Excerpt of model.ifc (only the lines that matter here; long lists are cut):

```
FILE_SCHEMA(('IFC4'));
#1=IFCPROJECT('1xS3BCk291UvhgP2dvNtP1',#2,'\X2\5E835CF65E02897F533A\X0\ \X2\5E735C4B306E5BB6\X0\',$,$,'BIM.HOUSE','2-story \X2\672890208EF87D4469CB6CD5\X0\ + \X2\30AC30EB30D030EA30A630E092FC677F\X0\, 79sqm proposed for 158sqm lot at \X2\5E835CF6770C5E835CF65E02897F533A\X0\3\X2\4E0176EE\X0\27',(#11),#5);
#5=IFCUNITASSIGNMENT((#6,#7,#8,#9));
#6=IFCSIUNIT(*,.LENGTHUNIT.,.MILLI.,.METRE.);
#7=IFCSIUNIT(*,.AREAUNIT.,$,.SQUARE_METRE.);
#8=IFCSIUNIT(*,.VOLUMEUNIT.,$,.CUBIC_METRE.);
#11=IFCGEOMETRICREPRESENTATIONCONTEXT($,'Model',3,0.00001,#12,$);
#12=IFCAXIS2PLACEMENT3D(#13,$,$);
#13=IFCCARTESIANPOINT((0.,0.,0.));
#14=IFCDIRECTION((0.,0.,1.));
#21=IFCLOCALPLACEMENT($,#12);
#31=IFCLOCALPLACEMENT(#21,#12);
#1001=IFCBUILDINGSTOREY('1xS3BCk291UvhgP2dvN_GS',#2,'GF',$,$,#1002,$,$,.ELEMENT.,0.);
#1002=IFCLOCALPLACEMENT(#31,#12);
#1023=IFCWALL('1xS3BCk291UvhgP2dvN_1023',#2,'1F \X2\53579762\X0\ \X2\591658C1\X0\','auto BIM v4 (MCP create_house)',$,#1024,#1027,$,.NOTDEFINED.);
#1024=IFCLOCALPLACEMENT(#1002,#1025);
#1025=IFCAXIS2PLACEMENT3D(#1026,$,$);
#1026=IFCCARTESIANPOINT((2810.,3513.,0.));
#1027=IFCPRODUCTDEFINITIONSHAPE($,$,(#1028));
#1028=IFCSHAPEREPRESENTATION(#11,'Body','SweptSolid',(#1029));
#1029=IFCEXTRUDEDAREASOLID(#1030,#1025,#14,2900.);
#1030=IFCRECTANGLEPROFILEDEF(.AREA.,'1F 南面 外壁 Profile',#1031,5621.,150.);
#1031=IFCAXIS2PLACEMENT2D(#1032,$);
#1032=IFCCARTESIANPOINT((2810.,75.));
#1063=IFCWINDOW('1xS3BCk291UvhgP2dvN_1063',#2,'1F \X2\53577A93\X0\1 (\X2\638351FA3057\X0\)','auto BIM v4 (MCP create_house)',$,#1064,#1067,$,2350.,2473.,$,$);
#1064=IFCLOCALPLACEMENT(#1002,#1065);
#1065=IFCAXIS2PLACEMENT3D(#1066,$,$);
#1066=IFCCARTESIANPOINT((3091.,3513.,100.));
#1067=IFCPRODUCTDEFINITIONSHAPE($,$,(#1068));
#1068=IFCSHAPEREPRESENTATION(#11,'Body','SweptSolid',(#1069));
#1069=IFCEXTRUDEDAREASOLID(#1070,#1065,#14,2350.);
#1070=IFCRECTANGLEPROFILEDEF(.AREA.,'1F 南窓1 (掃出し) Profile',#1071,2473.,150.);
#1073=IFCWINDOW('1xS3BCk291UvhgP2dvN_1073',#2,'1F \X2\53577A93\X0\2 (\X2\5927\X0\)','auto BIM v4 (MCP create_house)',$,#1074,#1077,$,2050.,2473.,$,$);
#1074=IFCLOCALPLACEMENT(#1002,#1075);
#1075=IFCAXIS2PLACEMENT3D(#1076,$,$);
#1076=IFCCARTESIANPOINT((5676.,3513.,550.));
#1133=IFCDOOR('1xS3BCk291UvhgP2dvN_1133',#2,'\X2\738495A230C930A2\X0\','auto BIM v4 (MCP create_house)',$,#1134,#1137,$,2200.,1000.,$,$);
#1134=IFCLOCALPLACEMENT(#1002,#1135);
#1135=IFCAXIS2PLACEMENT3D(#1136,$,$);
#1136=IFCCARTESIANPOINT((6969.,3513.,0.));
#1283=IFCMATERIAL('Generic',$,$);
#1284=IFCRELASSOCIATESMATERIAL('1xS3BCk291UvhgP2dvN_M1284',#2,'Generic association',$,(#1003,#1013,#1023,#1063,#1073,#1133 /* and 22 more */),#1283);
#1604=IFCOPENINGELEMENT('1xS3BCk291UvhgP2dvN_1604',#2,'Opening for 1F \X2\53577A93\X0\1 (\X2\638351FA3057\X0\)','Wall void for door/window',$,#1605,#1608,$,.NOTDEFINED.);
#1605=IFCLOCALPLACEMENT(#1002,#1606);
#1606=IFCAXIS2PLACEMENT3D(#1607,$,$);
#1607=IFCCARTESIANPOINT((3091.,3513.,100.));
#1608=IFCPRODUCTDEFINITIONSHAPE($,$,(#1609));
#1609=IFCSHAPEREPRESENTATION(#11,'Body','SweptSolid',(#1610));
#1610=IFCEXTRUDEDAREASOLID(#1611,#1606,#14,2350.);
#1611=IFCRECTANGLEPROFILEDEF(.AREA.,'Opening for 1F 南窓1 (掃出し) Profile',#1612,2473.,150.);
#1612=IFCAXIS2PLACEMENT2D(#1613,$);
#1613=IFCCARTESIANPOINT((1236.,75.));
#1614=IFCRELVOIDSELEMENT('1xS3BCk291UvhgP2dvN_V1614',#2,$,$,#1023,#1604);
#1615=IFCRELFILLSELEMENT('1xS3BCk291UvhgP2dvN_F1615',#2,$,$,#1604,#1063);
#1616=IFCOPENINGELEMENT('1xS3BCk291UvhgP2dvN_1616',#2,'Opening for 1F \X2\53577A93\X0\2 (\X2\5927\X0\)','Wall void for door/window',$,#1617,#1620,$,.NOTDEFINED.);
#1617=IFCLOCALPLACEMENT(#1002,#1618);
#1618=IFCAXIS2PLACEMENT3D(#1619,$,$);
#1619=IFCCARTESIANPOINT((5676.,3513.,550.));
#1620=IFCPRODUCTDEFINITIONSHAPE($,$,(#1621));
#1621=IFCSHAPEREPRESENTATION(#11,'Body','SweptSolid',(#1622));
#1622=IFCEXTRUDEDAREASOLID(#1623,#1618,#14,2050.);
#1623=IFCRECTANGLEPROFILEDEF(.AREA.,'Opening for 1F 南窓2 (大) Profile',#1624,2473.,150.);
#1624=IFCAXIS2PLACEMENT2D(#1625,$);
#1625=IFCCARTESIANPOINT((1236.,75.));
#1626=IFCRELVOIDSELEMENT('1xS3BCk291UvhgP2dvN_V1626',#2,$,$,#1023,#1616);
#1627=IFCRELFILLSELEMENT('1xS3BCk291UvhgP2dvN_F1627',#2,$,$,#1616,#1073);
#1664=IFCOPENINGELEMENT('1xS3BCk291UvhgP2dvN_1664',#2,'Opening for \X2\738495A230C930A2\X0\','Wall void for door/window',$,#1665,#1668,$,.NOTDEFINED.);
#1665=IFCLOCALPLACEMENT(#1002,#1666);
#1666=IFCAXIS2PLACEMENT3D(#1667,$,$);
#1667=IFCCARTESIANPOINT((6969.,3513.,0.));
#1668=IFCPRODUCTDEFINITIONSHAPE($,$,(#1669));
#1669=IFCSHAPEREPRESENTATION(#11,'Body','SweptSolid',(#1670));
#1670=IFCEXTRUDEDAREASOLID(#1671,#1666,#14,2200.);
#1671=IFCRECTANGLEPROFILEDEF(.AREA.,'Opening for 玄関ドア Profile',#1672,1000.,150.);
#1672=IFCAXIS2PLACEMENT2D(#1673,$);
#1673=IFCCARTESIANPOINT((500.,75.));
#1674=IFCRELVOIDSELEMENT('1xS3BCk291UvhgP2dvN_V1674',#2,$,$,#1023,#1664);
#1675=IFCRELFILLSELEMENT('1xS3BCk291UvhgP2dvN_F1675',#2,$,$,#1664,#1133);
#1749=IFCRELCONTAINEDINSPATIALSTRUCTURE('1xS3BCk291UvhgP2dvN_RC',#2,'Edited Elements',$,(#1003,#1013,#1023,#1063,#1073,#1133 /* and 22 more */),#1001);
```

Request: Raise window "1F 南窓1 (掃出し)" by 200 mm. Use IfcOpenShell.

```python
import numpy as np
import ifcopenshell
import ifcopenshell.api.geometry
import ifcopenshell.util.placement
import ifcopenshell.util.unit

model = ifcopenshell.open("model.ifc")
unit_scale = ifcopenshell.util.unit.calculate_unit_scale(model)

window = model.by_guid("1xS3BCk291UvhgP2dvN_1063")
opening = window.FillsVoids[0].RelatingOpeningElement
dz = 200.0

shift = np.array([0.0, 0.0, dz])
# The window is not placed relative to its opening, so move both.
for product in (opening, window):
    matrix = ifcopenshell.util.placement.get_local_placement(product.ObjectPlacement)
    matrix[:3, 3] += shift
    ifcopenshell.api.geometry.edit_object_placement(model, product=product, matrix=matrix, is_si=False)

print(f"moved by {dz * unit_scale:+.3f} m")

model.write("model_rev.ifc")
```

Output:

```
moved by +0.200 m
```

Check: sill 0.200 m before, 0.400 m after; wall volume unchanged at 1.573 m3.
